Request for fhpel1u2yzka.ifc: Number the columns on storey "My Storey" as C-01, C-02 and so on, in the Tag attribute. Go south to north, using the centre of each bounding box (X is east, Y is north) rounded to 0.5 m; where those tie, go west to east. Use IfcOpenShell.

First a look at what the model holds.

```python
import ifcopenshell
import ifcopenshell.util.element
import ifcopenshell.util.placement

model = ifcopenshell.open("fhpel1u2yzka.ifc")
print(model.schema)
storey = next(s for s in model.by_type("IfcBuildingStorey") if s.Name == "My Storey")
columns = [e for e in ifcopenshell.util.element.get_decomposition(storey) if e.is_a("IfcColumn")]
for e in sorted(columns, key=lambda e: e.id()):
    origin = ifcopenshell.util.placement.get_local_placement(e.ObjectPlacement)[:3, 3]
    print(e.id(), e.Tag, e.Name, origin.round(2) + 0.0, sep=" | ")
```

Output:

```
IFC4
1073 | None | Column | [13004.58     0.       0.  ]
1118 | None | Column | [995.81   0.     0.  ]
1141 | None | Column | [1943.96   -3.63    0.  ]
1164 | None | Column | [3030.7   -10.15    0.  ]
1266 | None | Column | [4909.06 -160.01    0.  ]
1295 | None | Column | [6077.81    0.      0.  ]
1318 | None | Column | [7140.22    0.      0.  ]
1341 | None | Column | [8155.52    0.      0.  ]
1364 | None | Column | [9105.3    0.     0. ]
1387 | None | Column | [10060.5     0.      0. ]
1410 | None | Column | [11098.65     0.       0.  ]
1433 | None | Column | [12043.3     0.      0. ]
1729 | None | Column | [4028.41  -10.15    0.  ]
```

```python
import ifcopenshell
import ifcopenshell.geom
import ifcopenshell.util.element
import ifcopenshell.util.shape

model = ifcopenshell.open("fhpel1u2yzka.ifc")
settings = ifcopenshell.geom.settings()
settings.set("use-world-coords", True)


def centre(element):
    shape = ifcopenshell.geom.create_shape(settings, element)
    return ifcopenshell.util.shape.get_bbox_centroid(shape.geometry)


storey = next(s for s in model.by_type("IfcBuildingStorey") if s.Name == "My Storey")
columns = [e for e in ifcopenshell.util.element.get_decomposition(storey) if e.is_a("IfcColumn")]

# Insertion points can sit at a corner or the storey origin, so sort by the geometry (in metres).
centres = {e: centre(e) for e in columns}
columns.sort(key=lambda e: (round(centres[e][1] / 0.5), centres[e][0]))

for i, e in enumerate(columns, start=1):
    number = f"C-{i:02d}"
    e.Tag = number
    print(e.id(), number)

model.write("fhpel1u2yzka_rev.ifc")
```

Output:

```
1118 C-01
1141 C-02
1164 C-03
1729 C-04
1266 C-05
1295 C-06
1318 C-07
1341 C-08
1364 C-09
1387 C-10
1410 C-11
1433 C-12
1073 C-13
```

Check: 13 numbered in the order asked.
